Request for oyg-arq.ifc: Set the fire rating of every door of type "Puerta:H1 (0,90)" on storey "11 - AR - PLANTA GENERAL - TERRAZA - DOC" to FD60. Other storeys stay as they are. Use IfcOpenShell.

First a look at what the model holds.

```python
import ifcopenshell
import ifcopenshell.util.element

model = ifcopenshell.open("oyg-arq.ifc")
print(model.schema)
storey = next(s for s in model.by_type("IfcBuildingStorey") if s.Name == "11 - AR - PLANTA GENERAL - TERRAZA - DOC")
doors = [e for e in ifcopenshell.util.element.get_decomposition(storey) if e.is_a("IfcDoor")]
seen = {}
for e in doors:
    element_type = ifcopenshell.util.element.get_type(e)
    key = (element_type.Name if element_type != e and element_type else None, ifcopenshell.util.element.get_pset(e, "Pset_DoorCommon", "FireRating"))
    seen[key] = seen.get(key, 0) + 1
for (name, value), count in sorted(seen.items(), key=str):
    print(count, "x", name, "|", value)
```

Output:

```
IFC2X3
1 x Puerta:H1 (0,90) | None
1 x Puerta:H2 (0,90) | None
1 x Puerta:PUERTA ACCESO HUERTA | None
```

```python
import ifcopenshell
import ifcopenshell.api.pset
import ifcopenshell.util.element

model = ifcopenshell.open("oyg-arq.ifc")

storey = next(s for s in model.by_type("IfcBuildingStorey") if s.Name == "11 - AR - PLANTA GENERAL - TERRAZA - DOC")
doors = [e for e in ifcopenshell.util.element.get_decomposition(storey) if e.is_a("IfcDoor")]

count = 0
for e in doors:
    element_type = ifcopenshell.util.element.get_type(e)
    if element_type in (None, e) or element_type.Name != "Puerta:H1 (0,90)":
        continue
    # add_pset returns the element's existing set when there is one.
    pset = ifcopenshell.api.pset.add_pset(model, product=e, name="Pset_DoorCommon")
    ifcopenshell.api.pset.edit_pset(model, pset=pset, properties={"FireRating": "FD60"})
    count += 1

print(count, "doors updated")

model.write("oyg-arq_updated.ifc")
```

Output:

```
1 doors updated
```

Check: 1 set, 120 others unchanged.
